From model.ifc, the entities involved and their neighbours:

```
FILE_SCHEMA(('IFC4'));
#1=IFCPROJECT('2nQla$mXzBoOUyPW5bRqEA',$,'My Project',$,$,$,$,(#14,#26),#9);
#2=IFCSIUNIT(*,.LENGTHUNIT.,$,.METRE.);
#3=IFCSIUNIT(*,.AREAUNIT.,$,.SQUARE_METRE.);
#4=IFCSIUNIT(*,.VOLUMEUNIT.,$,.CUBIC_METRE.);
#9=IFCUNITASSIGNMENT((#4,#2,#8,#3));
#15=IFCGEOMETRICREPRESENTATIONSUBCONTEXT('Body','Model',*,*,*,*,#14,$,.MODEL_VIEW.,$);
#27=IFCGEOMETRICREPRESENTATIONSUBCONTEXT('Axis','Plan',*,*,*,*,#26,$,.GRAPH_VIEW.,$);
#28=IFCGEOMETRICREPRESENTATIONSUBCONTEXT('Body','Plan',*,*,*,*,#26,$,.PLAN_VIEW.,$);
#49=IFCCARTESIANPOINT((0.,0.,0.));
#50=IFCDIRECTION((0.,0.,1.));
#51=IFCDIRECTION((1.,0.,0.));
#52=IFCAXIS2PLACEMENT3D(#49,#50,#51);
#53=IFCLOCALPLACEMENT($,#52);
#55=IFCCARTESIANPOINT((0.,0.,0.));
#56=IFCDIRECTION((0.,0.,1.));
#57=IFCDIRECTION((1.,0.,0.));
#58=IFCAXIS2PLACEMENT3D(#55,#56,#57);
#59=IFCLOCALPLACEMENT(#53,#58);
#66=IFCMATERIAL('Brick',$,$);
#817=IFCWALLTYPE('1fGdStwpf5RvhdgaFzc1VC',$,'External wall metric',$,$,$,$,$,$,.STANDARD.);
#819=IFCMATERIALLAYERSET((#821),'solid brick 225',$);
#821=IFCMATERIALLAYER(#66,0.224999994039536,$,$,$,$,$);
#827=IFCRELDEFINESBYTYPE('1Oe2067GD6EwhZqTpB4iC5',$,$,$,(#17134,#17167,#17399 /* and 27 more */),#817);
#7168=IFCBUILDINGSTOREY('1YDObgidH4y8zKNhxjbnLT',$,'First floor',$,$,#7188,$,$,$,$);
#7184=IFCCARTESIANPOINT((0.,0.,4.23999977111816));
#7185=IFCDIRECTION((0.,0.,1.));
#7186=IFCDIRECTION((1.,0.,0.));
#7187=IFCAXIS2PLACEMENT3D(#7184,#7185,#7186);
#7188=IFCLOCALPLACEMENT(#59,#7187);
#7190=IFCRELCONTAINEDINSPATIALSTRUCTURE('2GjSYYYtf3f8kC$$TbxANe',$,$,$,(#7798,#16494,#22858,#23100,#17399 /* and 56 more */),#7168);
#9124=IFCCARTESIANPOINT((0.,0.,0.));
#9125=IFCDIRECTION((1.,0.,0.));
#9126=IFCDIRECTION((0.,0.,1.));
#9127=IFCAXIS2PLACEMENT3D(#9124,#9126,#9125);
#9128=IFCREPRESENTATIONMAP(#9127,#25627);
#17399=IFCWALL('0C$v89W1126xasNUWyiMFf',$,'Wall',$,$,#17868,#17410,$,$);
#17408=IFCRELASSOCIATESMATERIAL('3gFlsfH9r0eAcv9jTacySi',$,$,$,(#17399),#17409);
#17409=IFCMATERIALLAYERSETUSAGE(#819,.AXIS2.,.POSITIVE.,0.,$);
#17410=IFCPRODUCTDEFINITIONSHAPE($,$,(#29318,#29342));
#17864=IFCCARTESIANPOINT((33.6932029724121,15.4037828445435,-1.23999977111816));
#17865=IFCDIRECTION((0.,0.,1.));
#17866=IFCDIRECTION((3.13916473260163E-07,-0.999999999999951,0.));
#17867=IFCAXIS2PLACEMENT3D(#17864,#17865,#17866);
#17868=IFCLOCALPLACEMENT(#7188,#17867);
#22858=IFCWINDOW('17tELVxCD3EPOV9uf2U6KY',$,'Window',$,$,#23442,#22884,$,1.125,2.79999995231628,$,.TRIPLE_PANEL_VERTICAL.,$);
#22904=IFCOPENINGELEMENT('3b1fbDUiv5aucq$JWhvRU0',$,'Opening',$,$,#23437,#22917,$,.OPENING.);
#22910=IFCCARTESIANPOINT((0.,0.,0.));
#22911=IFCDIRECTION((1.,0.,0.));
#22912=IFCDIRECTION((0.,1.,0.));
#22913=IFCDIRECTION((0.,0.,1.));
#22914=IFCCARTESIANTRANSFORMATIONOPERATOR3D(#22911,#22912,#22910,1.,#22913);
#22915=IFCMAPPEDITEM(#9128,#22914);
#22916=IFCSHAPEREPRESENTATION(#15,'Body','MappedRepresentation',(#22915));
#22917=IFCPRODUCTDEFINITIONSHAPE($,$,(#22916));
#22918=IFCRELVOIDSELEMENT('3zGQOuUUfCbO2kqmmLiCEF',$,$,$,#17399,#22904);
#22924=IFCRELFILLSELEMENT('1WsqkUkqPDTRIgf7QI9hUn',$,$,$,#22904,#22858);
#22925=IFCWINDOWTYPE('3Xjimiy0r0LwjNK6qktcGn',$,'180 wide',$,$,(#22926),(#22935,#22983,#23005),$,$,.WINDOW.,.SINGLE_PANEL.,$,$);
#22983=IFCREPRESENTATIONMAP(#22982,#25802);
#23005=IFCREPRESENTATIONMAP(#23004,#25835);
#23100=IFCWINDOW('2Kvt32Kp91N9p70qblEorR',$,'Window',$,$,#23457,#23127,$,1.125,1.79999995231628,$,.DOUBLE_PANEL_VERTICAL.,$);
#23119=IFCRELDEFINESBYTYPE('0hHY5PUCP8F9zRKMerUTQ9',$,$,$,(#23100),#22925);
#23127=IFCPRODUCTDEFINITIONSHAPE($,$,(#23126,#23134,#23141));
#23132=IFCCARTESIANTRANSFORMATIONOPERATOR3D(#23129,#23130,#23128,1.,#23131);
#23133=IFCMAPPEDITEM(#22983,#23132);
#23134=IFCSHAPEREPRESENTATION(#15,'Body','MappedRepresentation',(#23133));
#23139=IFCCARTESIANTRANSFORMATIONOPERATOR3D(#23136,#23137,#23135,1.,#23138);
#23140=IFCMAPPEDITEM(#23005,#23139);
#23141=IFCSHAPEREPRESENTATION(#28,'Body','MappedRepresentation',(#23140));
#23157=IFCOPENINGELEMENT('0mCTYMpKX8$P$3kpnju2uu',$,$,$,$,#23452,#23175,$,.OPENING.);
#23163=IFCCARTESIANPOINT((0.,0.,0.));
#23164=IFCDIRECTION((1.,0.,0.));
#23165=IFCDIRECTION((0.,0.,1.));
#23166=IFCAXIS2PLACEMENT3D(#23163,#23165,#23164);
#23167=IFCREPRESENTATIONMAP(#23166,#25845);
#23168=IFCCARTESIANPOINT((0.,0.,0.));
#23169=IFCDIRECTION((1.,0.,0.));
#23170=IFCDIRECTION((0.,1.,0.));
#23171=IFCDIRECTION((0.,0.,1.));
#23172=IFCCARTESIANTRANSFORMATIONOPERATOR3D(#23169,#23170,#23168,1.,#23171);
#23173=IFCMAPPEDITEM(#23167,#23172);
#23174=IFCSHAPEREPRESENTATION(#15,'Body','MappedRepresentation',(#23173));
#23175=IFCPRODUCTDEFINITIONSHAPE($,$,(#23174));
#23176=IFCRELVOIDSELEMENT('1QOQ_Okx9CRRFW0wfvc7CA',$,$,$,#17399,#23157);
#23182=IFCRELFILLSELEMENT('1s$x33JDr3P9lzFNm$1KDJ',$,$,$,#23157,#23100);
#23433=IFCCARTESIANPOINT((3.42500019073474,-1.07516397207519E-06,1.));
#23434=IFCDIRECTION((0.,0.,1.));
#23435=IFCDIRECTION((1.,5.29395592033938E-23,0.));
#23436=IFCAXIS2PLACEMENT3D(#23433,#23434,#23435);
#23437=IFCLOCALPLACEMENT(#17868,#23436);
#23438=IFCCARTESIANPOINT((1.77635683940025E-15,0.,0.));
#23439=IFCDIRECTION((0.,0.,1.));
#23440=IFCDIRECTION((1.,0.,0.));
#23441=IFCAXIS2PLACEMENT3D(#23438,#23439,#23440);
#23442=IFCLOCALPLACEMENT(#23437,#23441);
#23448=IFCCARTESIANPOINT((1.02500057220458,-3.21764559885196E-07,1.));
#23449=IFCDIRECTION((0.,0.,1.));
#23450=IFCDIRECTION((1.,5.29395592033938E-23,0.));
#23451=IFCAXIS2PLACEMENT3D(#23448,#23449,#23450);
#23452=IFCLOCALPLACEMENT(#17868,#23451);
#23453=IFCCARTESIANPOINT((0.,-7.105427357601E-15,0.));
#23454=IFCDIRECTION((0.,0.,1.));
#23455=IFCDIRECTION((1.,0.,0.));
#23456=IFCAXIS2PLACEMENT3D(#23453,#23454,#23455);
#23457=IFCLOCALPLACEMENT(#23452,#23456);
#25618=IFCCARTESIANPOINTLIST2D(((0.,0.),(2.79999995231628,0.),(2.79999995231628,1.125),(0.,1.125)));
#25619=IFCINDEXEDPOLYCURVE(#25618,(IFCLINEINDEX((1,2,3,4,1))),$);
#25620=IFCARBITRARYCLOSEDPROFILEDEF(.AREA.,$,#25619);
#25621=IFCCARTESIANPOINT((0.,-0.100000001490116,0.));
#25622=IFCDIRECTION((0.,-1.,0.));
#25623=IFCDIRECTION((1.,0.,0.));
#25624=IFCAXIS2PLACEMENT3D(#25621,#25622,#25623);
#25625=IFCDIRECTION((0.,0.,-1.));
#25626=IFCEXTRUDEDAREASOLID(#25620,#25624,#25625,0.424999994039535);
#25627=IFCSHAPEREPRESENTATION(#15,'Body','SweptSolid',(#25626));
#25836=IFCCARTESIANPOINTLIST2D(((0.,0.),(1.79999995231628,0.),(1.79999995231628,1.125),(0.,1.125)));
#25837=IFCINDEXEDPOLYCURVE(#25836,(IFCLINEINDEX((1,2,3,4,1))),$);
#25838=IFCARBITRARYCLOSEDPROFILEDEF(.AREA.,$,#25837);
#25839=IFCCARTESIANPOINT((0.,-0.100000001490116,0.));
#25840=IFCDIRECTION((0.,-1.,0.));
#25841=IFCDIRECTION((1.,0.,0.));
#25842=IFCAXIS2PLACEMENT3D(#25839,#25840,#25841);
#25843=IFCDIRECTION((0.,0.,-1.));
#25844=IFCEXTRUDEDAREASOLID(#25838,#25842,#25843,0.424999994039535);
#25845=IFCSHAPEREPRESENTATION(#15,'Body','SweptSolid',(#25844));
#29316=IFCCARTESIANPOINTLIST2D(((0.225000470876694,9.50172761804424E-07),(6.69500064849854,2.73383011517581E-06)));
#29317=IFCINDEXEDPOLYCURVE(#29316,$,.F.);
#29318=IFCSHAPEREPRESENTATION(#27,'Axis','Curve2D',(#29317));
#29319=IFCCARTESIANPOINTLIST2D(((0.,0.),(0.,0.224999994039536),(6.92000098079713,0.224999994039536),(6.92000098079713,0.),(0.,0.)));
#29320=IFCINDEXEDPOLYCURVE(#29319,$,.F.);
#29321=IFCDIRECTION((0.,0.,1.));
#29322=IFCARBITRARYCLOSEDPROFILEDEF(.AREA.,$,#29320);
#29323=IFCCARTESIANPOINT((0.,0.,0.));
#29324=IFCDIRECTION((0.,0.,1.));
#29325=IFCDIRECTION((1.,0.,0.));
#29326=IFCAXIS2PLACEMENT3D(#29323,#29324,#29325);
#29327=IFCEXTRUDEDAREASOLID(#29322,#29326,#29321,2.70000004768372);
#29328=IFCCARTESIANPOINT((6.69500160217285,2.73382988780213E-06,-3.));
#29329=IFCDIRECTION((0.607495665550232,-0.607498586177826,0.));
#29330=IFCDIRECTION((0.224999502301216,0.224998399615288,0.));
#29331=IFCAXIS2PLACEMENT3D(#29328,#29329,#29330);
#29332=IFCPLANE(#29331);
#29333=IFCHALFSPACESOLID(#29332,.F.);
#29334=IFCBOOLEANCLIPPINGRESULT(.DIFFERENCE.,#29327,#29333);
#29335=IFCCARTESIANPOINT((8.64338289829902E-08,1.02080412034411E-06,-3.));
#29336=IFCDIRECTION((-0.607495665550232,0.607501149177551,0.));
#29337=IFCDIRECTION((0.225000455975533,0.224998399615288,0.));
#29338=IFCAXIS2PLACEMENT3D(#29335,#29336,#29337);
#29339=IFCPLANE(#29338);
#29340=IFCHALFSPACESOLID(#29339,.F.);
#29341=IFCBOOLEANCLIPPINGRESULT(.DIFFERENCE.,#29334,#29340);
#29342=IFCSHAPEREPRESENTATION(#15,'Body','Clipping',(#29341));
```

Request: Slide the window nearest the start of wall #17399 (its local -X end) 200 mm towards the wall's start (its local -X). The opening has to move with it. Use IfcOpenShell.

```python
import ifcopenshell
import ifcopenshell.api.geometry
import ifcopenshell.util.placement
import ifcopenshell.util.unit

model = ifcopenshell.open("model.ifc")
unit_scale = ifcopenshell.util.unit.calculate_unit_scale(model)

window = model.by_guid("2Kvt32Kp91N9p70qblEorR")
opening = window.FillsVoids[0].RelatingOpeningElement
wall = opening.VoidsElements[0].RelatingBuildingElement

wall_matrix = ifcopenshell.util.placement.get_local_placement(wall.ObjectPlacement)
shift = wall_matrix[:3, 0] * -0.2 / unit_scale
before = ifcopenshell.util.placement.get_local_placement(window.ObjectPlacement)[:3, 3].copy()

# The window is placed relative to its opening, so it follows when the opening moves.
matrix = ifcopenshell.util.placement.get_local_placement(opening.ObjectPlacement)
matrix[:3, 3] += shift
ifcopenshell.api.geometry.edit_object_placement(
    model, product=opening, matrix=matrix, is_si=False, should_transform_children=True
)

after = ifcopenshell.util.placement.get_local_placement(window.ObjectPlacement)[:3, 3]
print("window moved by", (after - before).round(3) + 0.0)

model.write("model_edited.ifc")
```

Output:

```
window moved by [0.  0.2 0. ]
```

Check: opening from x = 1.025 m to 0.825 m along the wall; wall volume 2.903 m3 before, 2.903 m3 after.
